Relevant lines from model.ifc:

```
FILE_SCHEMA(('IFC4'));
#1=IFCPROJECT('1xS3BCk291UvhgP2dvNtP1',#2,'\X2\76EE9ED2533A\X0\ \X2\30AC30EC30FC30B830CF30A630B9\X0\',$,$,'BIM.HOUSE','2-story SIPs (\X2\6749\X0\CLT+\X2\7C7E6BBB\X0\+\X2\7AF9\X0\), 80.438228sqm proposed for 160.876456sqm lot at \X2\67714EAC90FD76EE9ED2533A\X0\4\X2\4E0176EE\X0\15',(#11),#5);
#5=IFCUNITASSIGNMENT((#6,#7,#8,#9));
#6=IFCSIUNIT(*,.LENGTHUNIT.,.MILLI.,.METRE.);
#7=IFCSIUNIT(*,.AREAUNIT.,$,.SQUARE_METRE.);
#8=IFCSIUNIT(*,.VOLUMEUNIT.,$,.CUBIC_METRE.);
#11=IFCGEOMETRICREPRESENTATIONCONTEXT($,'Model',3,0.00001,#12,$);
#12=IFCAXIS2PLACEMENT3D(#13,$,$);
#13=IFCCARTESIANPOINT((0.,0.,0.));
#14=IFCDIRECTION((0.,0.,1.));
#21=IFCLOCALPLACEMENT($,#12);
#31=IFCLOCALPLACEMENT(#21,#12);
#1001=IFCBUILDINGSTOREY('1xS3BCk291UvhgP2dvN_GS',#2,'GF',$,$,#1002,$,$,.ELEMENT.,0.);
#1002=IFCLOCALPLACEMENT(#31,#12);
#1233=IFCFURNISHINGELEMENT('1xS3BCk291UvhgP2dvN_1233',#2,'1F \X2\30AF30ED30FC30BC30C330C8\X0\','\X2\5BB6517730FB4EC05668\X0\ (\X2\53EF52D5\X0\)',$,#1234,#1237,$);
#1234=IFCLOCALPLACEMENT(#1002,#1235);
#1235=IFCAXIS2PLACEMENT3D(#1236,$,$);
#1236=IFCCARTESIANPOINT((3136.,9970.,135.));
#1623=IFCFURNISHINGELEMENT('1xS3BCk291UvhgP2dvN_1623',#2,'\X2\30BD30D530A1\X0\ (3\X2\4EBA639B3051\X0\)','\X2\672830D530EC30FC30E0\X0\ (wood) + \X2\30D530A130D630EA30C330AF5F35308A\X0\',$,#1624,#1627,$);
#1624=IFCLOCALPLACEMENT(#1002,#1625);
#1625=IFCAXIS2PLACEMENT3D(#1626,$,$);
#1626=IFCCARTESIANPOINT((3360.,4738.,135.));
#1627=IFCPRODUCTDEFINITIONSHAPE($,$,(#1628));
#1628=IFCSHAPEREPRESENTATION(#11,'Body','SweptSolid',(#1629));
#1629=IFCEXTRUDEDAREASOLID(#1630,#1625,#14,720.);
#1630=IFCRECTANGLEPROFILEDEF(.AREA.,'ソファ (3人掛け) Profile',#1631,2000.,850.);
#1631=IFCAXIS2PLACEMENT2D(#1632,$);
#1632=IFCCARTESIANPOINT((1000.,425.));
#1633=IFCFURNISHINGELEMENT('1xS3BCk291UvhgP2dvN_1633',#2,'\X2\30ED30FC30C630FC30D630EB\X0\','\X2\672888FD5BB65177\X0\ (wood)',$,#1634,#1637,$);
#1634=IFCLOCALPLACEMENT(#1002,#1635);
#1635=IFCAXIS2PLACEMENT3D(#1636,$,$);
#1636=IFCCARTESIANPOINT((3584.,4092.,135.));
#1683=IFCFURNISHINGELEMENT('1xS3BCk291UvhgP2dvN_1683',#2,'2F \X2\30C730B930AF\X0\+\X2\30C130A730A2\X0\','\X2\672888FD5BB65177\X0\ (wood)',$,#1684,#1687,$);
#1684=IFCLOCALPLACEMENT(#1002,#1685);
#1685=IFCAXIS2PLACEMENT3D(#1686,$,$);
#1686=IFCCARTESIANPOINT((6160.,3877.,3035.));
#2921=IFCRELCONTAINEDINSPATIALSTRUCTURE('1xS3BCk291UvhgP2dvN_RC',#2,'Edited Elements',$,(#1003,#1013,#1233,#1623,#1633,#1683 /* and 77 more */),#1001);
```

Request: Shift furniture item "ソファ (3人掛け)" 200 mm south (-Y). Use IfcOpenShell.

```python
import ifcopenshell
import ifcopenshell.api.geometry
import ifcopenshell.util.placement

model = ifcopenshell.open("model.ifc")

item = model.by_id(1623)
matrix = ifcopenshell.util.placement.get_local_placement(item.ObjectPlacement)
matrix[1, 3] -= 200.0
ifcopenshell.api.geometry.edit_object_placement(model, product=item, matrix=matrix, is_si=False)

print(ifcopenshell.util.placement.get_local_placement(item.ObjectPlacement).round(3) + 0.0)

model.write("model_edited.ifc")
```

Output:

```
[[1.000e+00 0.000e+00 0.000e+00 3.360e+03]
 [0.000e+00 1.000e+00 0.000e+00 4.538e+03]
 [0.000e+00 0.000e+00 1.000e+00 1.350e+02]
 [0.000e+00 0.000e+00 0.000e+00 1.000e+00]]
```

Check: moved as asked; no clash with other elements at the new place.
